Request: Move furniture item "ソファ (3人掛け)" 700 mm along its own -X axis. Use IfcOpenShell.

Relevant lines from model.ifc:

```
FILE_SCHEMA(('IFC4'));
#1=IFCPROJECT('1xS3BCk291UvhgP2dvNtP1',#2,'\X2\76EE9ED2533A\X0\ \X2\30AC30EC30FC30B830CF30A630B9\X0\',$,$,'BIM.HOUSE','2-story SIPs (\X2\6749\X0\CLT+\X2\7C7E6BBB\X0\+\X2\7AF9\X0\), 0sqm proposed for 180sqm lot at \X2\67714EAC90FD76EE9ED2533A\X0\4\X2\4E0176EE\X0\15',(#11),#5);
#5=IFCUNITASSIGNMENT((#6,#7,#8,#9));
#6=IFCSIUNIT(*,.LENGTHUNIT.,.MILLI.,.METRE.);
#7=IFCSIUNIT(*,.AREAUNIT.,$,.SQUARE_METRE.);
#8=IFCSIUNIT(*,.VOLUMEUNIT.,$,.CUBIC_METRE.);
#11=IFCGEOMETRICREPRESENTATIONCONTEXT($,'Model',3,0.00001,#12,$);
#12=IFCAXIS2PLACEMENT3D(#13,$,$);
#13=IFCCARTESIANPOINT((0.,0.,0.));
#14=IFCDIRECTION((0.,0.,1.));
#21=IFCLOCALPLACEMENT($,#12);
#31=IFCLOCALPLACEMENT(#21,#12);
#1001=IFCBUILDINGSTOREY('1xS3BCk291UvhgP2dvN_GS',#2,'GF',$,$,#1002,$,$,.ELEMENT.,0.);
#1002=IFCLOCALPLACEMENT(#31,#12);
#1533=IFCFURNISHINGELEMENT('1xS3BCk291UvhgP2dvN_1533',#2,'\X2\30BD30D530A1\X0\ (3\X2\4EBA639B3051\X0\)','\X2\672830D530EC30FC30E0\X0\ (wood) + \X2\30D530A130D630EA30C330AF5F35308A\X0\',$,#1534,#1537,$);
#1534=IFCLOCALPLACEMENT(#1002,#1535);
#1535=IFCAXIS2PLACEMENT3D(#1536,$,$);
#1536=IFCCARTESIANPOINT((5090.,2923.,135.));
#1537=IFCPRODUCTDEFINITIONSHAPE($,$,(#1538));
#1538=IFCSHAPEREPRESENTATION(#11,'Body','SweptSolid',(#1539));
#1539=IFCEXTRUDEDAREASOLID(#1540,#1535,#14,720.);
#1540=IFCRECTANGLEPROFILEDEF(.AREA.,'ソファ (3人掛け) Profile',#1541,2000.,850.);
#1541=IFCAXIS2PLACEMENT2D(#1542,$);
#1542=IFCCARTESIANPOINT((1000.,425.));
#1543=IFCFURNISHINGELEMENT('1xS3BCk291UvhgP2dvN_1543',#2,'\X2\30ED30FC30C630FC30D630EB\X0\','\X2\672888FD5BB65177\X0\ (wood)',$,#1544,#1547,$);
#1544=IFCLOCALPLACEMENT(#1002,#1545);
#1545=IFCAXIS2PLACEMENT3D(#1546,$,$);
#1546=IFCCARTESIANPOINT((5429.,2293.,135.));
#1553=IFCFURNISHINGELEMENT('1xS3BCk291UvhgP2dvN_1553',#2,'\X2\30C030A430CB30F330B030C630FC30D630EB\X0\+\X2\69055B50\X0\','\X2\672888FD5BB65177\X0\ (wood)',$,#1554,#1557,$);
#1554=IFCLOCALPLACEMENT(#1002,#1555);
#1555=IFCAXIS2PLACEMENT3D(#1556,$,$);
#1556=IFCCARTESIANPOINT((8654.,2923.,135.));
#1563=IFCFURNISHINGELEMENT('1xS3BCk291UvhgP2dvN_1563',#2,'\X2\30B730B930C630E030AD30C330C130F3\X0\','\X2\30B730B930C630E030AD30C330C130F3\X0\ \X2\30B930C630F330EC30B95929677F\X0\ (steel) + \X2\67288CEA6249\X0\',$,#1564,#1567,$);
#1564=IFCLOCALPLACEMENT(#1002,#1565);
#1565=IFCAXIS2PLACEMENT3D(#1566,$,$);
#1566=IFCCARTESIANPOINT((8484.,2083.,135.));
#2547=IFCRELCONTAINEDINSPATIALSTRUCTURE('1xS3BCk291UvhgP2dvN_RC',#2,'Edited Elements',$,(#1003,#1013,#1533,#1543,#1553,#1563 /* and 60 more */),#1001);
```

```python
import ifcopenshell
import ifcopenshell.api.geometry
import ifcopenshell.util.placement

model = ifcopenshell.open("model.ifc")

item = model.by_id(1533)
matrix = ifcopenshell.util.placement.get_local_placement(item.ObjectPlacement)
matrix[:3, 3] -= matrix[:3, 0] * 700.0
ifcopenshell.api.geometry.edit_object_placement(model, product=item, matrix=matrix, is_si=False)

print(ifcopenshell.util.placement.get_local_placement(item.ObjectPlacement).round(3) + 0.0)

model.write("model_v2.ifc")
```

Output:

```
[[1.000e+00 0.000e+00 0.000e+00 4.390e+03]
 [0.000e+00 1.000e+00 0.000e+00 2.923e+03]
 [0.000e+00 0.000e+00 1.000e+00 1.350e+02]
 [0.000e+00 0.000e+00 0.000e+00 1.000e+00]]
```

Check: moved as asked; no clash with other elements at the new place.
